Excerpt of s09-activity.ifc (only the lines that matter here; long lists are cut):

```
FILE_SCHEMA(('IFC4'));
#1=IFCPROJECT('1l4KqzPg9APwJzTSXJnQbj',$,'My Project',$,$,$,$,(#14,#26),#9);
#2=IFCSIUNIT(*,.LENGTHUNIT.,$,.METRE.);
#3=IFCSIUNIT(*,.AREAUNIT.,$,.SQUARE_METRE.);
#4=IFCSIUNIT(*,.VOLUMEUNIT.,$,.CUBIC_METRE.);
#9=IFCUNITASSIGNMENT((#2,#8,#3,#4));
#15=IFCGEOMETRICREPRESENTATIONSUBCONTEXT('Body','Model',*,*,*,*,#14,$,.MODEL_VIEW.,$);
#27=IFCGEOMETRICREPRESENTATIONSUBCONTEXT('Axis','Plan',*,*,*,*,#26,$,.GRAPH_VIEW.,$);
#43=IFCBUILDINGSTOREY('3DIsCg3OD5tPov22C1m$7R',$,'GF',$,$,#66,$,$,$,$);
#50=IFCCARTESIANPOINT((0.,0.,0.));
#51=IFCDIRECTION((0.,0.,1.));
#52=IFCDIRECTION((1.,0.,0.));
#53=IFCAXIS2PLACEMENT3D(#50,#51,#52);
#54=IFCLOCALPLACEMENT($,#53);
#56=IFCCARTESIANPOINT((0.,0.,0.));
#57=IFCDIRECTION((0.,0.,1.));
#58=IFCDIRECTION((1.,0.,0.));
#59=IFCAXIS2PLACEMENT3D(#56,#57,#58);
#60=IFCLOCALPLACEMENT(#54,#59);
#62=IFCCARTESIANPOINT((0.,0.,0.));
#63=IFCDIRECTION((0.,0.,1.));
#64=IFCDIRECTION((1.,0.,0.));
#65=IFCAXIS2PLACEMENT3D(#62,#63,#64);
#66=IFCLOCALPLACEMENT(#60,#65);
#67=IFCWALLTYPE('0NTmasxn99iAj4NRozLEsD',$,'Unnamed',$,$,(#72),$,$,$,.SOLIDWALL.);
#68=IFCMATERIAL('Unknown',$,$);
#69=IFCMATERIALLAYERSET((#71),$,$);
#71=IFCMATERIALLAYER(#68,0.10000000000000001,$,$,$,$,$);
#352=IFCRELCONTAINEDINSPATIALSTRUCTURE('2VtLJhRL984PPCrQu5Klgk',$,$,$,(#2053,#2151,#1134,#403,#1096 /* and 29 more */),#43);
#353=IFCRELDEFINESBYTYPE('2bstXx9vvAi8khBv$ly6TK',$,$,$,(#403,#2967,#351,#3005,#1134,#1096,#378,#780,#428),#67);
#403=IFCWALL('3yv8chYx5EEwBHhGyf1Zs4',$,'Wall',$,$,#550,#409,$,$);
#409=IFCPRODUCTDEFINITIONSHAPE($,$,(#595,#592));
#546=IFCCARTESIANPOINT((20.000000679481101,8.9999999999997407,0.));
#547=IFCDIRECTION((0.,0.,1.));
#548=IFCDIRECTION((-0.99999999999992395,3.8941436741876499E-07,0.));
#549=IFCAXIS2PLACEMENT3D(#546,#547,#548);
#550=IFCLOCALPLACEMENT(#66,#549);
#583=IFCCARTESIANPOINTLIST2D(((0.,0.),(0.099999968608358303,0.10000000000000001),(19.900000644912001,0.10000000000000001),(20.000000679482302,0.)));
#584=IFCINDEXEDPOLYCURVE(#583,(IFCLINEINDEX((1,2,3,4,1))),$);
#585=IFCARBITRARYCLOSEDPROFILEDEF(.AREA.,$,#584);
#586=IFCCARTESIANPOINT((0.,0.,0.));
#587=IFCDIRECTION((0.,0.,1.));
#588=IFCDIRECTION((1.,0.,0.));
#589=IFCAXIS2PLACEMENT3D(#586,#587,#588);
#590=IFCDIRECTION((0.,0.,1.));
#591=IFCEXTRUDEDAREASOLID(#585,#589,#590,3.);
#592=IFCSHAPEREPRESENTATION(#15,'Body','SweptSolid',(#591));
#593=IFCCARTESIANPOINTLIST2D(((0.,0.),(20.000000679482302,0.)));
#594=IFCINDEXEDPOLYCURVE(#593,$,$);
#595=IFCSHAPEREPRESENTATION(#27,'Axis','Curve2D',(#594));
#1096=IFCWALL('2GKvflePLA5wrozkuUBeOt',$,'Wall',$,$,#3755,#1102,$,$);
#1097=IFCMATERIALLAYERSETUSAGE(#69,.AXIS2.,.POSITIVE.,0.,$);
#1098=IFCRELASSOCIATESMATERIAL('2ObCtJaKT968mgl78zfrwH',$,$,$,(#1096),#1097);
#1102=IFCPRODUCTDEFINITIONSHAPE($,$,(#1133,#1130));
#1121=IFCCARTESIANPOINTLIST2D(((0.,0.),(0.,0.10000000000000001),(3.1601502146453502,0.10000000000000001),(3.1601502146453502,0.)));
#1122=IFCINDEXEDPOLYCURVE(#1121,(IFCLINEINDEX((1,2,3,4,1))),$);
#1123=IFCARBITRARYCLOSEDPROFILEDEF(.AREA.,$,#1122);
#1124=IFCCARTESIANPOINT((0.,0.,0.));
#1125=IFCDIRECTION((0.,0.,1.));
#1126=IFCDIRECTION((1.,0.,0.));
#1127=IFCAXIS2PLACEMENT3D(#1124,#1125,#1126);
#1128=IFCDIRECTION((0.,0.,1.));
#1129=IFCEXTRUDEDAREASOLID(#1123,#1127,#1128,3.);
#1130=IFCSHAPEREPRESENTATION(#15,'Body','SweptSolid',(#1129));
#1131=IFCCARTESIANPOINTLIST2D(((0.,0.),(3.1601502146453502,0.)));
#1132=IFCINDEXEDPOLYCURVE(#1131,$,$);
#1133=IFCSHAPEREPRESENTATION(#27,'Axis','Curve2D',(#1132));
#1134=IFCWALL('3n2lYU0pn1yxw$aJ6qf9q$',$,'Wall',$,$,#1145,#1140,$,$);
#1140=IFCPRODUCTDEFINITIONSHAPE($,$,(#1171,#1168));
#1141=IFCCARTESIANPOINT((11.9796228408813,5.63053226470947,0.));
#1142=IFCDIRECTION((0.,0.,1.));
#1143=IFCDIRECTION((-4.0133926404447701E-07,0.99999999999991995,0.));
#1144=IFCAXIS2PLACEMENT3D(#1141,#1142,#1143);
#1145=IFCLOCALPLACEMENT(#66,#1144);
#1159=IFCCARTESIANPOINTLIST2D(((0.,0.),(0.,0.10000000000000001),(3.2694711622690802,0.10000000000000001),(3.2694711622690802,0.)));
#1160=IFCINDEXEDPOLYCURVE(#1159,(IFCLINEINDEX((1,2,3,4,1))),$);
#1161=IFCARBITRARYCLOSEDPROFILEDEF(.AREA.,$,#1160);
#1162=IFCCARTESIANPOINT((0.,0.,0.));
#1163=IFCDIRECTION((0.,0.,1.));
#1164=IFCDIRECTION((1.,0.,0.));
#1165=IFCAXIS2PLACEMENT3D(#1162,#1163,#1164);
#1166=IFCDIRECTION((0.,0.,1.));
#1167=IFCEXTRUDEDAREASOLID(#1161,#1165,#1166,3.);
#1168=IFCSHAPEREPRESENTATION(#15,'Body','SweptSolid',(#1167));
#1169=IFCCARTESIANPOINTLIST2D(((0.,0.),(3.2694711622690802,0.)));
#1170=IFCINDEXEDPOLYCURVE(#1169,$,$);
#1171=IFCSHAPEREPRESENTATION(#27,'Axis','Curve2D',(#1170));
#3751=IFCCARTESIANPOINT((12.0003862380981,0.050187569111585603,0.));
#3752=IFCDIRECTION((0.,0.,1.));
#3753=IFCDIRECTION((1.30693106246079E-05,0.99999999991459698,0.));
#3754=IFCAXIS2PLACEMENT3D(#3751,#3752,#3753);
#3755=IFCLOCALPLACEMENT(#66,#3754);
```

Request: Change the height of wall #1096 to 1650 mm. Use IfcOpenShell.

```python
import ifcopenshell
import ifcopenshell.geom
import ifcopenshell.util.representation
import ifcopenshell.util.shape
import ifcopenshell.util.unit

model = ifcopenshell.open("s09-activity.ifc")
unit_scale = ifcopenshell.util.unit.calculate_unit_scale(model)
settings = ifcopenshell.geom.settings()


def volume(element):
    """Net volume in cubic metres, openings subtracted."""
    shape = ifcopenshell.geom.create_shape(settings, element)
    return ifcopenshell.util.shape.get_volume(shape.geometry)


wall = model.by_guid("2GKvflePLA5wrozkuUBeOt")
before = volume(wall)

body = ifcopenshell.util.representation.get_representation(wall, "Model", "Body")
solid = body.Items[0]
old_height = solid.Depth
solid.Depth = 1.65 / unit_scale
after = volume(wall)

print(f"height {old_height:g} -> {solid.Depth:g}, volume {before:.3f} -> {after:.3f} m3")

model.write("s09-activity_rev.ifc")
```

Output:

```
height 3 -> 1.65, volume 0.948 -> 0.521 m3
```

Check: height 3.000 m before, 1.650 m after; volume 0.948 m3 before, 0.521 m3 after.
